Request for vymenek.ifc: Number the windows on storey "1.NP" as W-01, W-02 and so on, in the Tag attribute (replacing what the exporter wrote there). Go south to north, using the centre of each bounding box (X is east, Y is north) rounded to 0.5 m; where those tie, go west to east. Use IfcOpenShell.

First a look at what the model holds.

```python
import ifcopenshell
import ifcopenshell.util.element
import ifcopenshell.util.placement

model = ifcopenshell.open("vymenek.ifc")
print(model.schema)
storey = next(s for s in model.by_type("IfcBuildingStorey") if s.Name == "1.NP")
windows = [e for e in ifcopenshell.util.element.get_decomposition(storey) if e.is_a("IfcWindow")]
for e in sorted(windows, key=lambda e: e.id()):
    origin = ifcopenshell.util.placement.get_local_placement(e.ObjectPlacement)[:3, 3]
    print(e.id(), e.Tag, e.Name, origin.round(2) + 0.0, sep=" | ")
```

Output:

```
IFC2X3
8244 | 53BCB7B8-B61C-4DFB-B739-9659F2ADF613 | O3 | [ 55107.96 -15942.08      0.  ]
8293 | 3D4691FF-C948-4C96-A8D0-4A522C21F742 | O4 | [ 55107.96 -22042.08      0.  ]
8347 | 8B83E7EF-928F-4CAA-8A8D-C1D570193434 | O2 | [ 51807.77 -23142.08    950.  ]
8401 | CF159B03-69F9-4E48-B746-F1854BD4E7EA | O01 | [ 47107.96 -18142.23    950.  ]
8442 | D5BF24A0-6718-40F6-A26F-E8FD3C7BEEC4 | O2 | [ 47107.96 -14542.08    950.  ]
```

```python
import ifcopenshell
import ifcopenshell.geom
import ifcopenshell.util.element
import ifcopenshell.util.shape

model = ifcopenshell.open("vymenek.ifc")
settings = ifcopenshell.geom.settings()
settings.set("use-world-coords", True)


def centre(element):
    shape = ifcopenshell.geom.create_shape(settings, element)
    return ifcopenshell.util.shape.get_bbox_centroid(shape.geometry)


storey = next(s for s in model.by_type("IfcBuildingStorey") if s.Name == "1.NP")
windows = [e for e in ifcopenshell.util.element.get_decomposition(storey) if e.is_a("IfcWindow")]

# Insertion points can sit at a corner or the storey origin, so sort by the geometry (in metres).
centres = {e: centre(e) for e in windows}
windows.sort(key=lambda e: (round(centres[e][1] / 0.5), centres[e][0]))

for i, e in enumerate(windows, start=1):
    number = f"W-{i:02d}"
    e.Tag = number
    print(e.id(), number)

model.write("vymenek-out.ifc")
```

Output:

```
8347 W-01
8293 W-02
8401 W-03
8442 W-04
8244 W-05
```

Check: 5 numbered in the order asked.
